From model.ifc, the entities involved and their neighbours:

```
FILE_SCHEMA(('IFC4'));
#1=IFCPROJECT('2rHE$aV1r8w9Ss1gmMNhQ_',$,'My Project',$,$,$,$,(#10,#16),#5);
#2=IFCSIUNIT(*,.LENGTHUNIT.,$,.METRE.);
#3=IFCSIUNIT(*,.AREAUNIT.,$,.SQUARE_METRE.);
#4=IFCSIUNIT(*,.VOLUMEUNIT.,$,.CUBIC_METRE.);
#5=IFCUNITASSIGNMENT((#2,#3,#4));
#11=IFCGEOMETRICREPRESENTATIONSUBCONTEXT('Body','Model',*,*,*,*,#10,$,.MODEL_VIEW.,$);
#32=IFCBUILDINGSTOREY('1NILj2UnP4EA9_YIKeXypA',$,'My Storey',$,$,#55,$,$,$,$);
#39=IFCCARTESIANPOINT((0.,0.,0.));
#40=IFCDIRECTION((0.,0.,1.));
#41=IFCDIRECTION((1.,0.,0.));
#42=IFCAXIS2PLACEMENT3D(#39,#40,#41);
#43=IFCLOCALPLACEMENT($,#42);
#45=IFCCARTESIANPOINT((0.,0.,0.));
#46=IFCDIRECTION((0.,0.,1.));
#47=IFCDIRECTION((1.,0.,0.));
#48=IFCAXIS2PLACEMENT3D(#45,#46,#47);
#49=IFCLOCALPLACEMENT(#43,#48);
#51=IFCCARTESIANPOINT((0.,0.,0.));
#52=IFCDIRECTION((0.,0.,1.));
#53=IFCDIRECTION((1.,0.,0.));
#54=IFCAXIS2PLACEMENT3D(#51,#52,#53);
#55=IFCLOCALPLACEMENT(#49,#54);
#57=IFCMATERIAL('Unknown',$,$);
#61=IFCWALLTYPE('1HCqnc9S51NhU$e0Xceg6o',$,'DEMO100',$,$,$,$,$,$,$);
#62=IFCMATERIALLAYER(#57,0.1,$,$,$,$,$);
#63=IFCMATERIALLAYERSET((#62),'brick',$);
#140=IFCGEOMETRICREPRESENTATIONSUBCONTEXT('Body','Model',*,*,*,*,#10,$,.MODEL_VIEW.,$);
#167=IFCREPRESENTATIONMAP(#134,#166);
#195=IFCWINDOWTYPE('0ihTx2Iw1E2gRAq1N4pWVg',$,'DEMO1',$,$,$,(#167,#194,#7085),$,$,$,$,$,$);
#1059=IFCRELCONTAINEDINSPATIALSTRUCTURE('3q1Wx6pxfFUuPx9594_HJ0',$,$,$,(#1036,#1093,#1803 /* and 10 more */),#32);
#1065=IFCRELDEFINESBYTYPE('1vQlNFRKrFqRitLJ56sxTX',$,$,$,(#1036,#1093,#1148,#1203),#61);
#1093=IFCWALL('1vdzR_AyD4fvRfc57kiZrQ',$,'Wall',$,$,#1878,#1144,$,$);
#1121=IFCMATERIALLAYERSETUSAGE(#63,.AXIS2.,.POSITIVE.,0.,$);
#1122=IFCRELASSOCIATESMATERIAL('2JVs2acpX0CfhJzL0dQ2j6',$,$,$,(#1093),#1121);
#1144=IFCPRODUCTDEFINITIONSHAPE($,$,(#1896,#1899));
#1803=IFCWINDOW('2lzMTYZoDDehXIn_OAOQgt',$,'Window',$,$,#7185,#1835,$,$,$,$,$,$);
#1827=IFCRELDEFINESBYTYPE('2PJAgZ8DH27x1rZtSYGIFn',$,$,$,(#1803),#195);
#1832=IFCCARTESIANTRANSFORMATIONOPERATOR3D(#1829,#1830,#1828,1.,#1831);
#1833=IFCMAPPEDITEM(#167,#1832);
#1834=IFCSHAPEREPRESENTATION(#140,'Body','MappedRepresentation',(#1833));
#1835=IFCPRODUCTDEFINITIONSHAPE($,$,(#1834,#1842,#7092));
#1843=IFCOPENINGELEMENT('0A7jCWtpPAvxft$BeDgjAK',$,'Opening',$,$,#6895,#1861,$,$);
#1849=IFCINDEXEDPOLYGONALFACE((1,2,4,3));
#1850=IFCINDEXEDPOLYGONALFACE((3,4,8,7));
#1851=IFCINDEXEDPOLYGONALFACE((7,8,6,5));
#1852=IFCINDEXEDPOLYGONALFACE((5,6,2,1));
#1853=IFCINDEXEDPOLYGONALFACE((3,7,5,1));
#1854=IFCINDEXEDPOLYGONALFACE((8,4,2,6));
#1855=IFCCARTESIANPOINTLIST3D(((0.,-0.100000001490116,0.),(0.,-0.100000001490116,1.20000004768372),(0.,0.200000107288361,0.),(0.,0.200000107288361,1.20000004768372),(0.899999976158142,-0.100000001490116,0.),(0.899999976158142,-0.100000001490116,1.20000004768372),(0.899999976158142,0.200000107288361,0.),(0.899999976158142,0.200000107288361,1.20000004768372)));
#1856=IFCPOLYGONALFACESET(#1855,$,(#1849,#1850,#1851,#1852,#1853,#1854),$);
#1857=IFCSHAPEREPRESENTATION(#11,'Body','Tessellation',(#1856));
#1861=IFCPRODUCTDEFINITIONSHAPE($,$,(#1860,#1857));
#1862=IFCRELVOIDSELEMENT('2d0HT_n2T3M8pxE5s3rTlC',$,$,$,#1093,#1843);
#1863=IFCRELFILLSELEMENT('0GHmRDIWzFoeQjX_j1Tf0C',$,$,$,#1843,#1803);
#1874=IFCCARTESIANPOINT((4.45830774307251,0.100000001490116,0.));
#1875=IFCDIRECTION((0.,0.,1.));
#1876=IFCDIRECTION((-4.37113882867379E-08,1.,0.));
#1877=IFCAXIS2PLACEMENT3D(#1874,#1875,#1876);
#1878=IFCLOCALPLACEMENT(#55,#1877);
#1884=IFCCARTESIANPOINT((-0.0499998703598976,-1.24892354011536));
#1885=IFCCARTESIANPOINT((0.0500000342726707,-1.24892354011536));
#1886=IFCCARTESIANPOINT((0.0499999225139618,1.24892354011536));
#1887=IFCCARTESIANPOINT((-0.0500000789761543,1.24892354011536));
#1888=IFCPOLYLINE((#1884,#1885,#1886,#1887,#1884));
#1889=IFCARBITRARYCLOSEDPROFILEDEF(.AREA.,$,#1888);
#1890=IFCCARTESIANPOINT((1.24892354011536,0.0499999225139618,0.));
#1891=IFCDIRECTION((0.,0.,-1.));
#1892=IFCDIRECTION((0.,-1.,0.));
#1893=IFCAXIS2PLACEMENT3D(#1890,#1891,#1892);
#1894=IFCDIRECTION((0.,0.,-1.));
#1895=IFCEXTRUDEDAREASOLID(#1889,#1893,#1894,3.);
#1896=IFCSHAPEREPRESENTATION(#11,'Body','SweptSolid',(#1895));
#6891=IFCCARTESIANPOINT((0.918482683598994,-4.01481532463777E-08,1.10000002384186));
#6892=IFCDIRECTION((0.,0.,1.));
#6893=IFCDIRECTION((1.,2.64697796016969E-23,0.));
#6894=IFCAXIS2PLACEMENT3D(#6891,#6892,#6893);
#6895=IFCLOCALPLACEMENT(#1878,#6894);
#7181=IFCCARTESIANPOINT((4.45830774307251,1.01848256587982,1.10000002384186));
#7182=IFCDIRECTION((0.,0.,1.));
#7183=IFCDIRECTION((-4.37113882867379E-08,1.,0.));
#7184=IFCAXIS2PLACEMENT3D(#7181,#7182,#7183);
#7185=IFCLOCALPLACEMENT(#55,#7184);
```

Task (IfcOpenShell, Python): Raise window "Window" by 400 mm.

```python
import numpy as np
import ifcopenshell
import ifcopenshell.api.geometry
import ifcopenshell.util.placement
import ifcopenshell.util.unit

model = ifcopenshell.open("model.ifc")
unit_scale = ifcopenshell.util.unit.calculate_unit_scale(model)

window = model.by_id(1803)
opening = window.FillsVoids[0].RelatingOpeningElement
dz = 0.4

shift = np.array([0.0, 0.0, dz])
# The window is not placed relative to its opening, so move both.
for product in (opening, window):
    matrix = ifcopenshell.util.placement.get_local_placement(product.ObjectPlacement)
    matrix[:3, 3] += shift
    ifcopenshell.api.geometry.edit_object_placement(model, product=product, matrix=matrix, is_si=False)

print(f"moved by {dz * unit_scale:+.3f} m")

model.write("model_edited.ifc")
```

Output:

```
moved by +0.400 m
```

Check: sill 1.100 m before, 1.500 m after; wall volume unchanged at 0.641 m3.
